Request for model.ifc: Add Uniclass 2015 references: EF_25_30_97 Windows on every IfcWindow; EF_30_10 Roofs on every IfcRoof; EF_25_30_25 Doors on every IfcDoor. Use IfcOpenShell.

First a look at what the model holds.

```python
import ifcopenshell

model = ifcopenshell.open("model.ifc")
print(model.schema)
print("classifications:", [c.Name for c in model.by_type("IfcClassification")])
for ifc_class in ("IfcDoor", "IfcRoof", "IfcStair", "IfcWall", "IfcWindow"):
    print(ifc_class, len(model.by_type(ifc_class)))
```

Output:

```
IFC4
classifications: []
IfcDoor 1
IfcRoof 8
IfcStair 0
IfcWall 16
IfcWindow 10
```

```python
import ifcopenshell
import ifcopenshell.api.classification

model = ifcopenshell.open("model.ifc")

system = ifcopenshell.api.classification.add_classification(model, classification="Uniclass 2015")

codes = {
    "IfcWindow": ("EF_25_30_97", "Windows"),
    "IfcRoof": ("EF_30_10", "Roofs"),
    "IfcDoor": ("EF_25_30_25", "Doors"),
}
for ifc_class, (code, name) in codes.items():
    products = model.by_type(ifc_class)
    ifcopenshell.api.classification.add_reference(
        model, products=products, classification=system, identification=code, name=name
    )
    print(code, len(products))

model.write("model-out.ifc")
```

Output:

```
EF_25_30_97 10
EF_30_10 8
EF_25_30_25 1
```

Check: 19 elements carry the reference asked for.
